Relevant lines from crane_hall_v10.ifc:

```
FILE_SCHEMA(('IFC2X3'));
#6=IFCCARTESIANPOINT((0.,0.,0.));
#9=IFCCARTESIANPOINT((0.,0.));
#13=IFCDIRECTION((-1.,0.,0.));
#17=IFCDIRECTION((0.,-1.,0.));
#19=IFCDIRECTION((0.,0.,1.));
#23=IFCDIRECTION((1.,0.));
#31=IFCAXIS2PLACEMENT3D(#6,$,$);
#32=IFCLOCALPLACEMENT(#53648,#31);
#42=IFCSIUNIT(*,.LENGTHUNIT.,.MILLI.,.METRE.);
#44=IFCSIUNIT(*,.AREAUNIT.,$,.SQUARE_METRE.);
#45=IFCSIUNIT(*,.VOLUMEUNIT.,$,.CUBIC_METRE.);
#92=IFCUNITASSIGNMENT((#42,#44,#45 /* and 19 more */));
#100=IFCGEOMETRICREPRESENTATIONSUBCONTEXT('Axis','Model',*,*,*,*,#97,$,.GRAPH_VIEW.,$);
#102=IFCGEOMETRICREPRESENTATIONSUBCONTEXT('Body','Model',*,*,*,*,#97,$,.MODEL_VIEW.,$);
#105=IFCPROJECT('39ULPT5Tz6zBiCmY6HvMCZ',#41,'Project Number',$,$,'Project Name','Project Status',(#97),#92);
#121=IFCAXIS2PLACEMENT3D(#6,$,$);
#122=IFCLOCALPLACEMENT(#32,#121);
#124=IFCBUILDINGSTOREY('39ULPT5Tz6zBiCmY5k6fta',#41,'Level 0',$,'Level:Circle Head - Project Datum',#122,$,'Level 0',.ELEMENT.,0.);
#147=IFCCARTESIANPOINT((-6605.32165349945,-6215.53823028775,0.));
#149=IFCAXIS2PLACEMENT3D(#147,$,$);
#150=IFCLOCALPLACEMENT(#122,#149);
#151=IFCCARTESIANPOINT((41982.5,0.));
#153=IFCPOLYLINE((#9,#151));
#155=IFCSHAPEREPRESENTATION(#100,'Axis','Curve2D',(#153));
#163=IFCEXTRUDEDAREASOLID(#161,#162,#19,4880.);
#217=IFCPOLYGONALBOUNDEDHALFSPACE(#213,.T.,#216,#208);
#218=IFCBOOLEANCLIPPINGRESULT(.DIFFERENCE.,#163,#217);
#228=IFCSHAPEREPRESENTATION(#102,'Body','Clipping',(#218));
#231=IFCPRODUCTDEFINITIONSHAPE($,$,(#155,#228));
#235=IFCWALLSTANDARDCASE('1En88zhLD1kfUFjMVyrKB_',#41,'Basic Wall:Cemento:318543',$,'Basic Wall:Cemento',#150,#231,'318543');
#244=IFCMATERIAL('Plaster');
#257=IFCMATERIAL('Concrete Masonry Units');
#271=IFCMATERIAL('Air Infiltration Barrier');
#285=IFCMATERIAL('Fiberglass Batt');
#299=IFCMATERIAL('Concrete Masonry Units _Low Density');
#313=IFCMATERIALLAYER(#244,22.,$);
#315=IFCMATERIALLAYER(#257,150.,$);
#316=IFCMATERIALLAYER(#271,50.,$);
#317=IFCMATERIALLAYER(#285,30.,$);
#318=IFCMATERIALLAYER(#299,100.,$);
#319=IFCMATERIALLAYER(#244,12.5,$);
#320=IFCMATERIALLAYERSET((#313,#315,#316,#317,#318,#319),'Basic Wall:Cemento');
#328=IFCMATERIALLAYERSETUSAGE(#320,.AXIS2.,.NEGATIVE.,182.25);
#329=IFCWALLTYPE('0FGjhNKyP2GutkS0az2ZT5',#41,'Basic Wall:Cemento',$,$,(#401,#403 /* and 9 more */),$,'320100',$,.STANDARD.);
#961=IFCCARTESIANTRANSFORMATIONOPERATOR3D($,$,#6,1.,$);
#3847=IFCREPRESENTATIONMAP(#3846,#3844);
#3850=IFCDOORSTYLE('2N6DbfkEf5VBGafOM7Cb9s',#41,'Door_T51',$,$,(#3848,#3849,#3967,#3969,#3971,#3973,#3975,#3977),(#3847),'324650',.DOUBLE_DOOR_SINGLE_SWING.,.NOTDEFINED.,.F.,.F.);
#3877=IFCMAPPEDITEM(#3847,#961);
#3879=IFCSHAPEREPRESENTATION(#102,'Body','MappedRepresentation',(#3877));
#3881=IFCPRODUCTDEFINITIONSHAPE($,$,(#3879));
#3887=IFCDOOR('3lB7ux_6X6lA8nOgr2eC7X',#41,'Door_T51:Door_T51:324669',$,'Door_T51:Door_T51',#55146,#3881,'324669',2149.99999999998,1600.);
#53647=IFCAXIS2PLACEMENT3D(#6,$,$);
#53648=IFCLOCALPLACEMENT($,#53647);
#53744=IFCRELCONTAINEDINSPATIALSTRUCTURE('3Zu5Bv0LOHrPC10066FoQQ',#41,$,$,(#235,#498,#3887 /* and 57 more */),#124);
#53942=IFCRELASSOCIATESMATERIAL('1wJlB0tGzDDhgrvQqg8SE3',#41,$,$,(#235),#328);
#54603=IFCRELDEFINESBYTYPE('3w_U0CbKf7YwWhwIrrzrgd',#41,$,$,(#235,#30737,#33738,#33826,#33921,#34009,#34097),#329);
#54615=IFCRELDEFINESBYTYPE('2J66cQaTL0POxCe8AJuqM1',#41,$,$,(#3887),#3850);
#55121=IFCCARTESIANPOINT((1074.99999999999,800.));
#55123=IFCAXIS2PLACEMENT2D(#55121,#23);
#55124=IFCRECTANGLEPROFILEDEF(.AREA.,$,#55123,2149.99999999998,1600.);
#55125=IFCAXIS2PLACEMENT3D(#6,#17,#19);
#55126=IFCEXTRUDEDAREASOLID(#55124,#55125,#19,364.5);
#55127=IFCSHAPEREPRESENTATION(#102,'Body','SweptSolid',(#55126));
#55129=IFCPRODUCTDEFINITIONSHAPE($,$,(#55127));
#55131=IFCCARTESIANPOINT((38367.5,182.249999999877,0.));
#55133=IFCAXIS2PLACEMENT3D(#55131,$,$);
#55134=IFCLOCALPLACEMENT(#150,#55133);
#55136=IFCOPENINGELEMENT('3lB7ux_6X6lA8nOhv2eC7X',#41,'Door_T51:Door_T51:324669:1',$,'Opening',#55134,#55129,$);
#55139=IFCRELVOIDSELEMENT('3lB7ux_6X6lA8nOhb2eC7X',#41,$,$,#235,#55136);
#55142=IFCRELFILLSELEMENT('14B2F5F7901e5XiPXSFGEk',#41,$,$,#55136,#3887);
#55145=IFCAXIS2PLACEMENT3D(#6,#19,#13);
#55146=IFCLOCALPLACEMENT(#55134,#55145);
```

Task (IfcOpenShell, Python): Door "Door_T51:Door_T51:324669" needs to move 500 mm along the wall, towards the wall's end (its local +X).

```python
import ifcopenshell
import ifcopenshell.api.geometry
import ifcopenshell.util.placement
import ifcopenshell.util.unit

model = ifcopenshell.open("crane_hall_v10.ifc")
unit_scale = ifcopenshell.util.unit.calculate_unit_scale(model)

door = model.by_guid("3lB7ux_6X6lA8nOgr2eC7X")
opening = door.FillsVoids[0].RelatingOpeningElement
wall = opening.VoidsElements[0].RelatingBuildingElement

wall_matrix = ifcopenshell.util.placement.get_local_placement(wall.ObjectPlacement)
shift = wall_matrix[:3, 0] * 0.5 / unit_scale
before = ifcopenshell.util.placement.get_local_placement(door.ObjectPlacement)[:3, 3].copy()

# The door is placed relative to its opening, so it follows when the opening moves.
matrix = ifcopenshell.util.placement.get_local_placement(opening.ObjectPlacement)
matrix[:3, 3] += shift
ifcopenshell.api.geometry.edit_object_placement(
    model, product=opening, matrix=matrix, is_si=False, should_transform_children=True
)

after = ifcopenshell.util.placement.get_local_placement(door.ObjectPlacement)[:3, 3]
print("door moved by", (after - before).round(3) + 0.0)

model.write("crane_hall_v10_edited.ifc")
```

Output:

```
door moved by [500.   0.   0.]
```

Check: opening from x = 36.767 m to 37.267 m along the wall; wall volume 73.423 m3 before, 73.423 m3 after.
